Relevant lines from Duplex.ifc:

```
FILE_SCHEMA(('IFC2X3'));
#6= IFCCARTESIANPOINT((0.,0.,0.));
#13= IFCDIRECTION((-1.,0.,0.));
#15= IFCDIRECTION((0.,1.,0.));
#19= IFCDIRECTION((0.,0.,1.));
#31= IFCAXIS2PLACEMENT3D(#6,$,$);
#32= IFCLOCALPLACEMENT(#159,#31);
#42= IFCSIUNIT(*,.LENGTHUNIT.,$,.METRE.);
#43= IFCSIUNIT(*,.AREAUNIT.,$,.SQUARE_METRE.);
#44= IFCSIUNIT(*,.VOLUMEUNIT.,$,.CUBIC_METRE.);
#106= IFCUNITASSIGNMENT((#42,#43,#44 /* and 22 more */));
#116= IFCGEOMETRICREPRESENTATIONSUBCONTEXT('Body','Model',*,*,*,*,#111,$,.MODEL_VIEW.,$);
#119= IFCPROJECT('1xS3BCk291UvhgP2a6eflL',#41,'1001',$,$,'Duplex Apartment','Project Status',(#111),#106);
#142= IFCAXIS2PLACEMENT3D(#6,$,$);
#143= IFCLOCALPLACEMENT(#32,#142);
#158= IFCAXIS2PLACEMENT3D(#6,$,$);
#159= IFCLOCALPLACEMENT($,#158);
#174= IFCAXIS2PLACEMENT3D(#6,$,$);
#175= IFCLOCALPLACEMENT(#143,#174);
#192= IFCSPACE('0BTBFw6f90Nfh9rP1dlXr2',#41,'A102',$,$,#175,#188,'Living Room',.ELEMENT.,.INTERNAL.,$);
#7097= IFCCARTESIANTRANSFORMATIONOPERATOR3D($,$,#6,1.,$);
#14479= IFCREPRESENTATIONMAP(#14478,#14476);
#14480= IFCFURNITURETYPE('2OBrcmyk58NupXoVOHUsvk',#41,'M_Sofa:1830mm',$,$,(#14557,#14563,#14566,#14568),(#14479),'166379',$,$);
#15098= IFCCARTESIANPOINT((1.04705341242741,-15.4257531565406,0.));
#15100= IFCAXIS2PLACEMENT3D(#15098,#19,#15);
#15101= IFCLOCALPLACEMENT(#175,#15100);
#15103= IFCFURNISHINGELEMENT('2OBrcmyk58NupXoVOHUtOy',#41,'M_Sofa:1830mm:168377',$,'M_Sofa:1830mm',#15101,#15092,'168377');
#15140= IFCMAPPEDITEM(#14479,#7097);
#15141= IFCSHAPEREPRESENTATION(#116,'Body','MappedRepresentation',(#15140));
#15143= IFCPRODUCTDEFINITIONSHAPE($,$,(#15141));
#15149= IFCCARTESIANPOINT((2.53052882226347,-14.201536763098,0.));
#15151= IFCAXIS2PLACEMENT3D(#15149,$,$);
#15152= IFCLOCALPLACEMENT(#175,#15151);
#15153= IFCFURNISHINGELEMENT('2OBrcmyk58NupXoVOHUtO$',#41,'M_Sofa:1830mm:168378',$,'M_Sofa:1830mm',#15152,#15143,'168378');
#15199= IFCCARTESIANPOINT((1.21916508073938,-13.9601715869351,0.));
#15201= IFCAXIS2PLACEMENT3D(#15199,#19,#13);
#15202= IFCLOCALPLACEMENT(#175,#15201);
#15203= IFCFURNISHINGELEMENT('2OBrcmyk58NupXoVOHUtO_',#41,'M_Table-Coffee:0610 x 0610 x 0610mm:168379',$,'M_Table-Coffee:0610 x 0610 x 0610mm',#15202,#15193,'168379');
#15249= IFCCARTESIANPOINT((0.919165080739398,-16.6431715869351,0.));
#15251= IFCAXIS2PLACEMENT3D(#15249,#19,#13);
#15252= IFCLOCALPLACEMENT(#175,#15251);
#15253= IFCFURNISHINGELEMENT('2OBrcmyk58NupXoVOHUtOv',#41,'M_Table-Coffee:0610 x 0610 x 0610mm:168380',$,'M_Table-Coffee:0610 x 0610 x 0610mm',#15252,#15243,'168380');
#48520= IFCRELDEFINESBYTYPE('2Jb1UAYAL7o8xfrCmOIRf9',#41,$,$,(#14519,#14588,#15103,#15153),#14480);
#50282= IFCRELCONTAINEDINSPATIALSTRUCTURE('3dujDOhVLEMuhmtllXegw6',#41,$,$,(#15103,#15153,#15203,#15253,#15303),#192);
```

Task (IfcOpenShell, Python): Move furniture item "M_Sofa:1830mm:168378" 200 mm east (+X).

```python
import ifcopenshell
import ifcopenshell.api.geometry
import ifcopenshell.util.placement
import ifcopenshell.util.unit

model = ifcopenshell.open("Duplex.ifc")
unit_scale = ifcopenshell.util.unit.calculate_unit_scale(model)

item = model.by_id(15153)
matrix = ifcopenshell.util.placement.get_local_placement(item.ObjectPlacement)
matrix[0, 3] += 0.2 / unit_scale
ifcopenshell.api.geometry.edit_object_placement(model, product=item, matrix=matrix, is_si=False)

print(ifcopenshell.util.placement.get_local_placement(item.ObjectPlacement).round(3) + 0.0)

model.write("Duplex_updated.ifc")
```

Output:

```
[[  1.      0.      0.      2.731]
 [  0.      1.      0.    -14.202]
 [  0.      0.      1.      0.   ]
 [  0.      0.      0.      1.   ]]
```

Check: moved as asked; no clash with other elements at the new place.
